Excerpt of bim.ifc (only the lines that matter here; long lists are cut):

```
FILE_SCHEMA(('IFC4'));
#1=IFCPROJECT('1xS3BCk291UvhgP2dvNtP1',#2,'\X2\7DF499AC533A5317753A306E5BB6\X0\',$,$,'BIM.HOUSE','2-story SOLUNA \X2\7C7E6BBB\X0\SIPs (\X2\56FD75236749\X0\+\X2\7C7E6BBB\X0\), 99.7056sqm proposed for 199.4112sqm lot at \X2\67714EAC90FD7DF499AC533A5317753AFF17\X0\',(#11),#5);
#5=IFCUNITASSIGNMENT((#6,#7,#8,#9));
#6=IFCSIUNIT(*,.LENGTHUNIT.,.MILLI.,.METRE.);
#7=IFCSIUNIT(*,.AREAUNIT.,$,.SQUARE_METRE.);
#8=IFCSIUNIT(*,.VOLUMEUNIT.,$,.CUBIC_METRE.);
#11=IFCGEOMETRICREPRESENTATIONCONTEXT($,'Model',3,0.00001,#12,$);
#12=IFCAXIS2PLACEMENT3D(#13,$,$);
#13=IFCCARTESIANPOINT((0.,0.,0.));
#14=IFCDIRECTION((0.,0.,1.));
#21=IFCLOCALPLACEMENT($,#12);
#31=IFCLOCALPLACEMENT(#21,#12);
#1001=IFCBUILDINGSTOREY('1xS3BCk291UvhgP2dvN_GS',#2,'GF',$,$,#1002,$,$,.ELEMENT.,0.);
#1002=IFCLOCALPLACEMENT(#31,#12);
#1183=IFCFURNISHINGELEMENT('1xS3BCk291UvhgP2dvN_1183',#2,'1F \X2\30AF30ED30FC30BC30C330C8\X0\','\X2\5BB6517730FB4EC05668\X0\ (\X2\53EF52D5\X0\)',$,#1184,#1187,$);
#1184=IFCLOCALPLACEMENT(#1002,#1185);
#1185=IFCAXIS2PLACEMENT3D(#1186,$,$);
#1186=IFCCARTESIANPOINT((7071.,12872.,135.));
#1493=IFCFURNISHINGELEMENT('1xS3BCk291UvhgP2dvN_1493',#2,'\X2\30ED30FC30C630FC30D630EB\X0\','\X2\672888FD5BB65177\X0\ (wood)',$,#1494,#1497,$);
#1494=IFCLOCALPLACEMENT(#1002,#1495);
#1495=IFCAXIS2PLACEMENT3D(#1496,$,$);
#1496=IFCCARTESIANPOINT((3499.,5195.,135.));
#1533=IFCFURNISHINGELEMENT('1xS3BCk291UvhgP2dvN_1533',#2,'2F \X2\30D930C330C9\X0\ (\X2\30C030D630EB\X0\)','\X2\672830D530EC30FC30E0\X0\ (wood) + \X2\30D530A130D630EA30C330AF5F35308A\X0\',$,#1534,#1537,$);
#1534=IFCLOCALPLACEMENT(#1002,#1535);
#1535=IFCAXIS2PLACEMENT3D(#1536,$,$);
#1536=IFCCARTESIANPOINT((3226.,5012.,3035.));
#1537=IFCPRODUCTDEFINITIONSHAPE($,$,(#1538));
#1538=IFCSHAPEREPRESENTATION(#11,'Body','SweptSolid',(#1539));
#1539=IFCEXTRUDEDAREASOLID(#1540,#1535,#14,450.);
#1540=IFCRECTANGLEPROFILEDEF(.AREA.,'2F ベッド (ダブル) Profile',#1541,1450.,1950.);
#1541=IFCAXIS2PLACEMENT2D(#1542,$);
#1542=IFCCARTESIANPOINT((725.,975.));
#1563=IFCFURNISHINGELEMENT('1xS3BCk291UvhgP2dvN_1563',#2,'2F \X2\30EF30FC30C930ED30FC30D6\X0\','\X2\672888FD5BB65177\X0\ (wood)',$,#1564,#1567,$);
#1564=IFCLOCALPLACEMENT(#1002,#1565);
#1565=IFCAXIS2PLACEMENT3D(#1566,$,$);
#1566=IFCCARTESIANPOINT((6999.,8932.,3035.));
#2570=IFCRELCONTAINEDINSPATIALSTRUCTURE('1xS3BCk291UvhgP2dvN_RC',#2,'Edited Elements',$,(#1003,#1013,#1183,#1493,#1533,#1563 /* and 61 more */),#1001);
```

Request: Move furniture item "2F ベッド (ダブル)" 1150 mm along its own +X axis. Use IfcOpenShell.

```python
import ifcopenshell
import ifcopenshell.api.geometry
import ifcopenshell.util.placement
import ifcopenshell.util.unit

model = ifcopenshell.open("bim.ifc")
unit_scale = ifcopenshell.util.unit.calculate_unit_scale(model)

item = model.by_guid("1xS3BCk291UvhgP2dvN_1533")
matrix = ifcopenshell.util.placement.get_local_placement(item.ObjectPlacement)
matrix[:3, 3] += matrix[:3, 0] * 1.15 / unit_scale
ifcopenshell.api.geometry.edit_object_placement(model, product=item, matrix=matrix, is_si=False)

print(ifcopenshell.util.placement.get_local_placement(item.ObjectPlacement).round(3) + 0.0)

model.write("bim_updated.ifc")
```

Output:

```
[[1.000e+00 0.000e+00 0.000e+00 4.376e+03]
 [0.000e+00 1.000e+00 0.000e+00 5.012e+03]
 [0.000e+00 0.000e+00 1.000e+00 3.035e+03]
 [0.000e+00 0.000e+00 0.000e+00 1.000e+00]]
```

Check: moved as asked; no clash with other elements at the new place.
